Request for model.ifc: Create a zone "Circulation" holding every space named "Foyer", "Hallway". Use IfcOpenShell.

First a look at what the model holds.

```python
import ifcopenshell

model = ifcopenshell.open("model.ifc")
print(model.schema)
seen = {}
for space in model.by_type("IfcSpace"):
    seen[space.LongName] = seen.get(space.LongName, 0) + 1
for name, count in sorted(seen.items(), key=str):
    print(count, "x", name)
print("zones:", [z.Name for z in model.by_type("IfcZone")][:20])
```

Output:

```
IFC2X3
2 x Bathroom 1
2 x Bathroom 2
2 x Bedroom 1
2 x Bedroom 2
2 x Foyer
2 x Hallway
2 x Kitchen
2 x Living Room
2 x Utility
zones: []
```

```python
import ifcopenshell
import ifcopenshell.api.group
import ifcopenshell.api.root

model = ifcopenshell.open("model.ifc")

names = {"Foyer", "Hallway"}
spaces = [s for s in model.by_type("IfcSpace") if s.LongName in names]

zone = ifcopenshell.api.root.create_entity(model, ifc_class="IfcZone", name="Circulation")
ifcopenshell.api.group.assign_group(model, products=spaces, group=zone)
print(len(spaces), "spaces in", zone.Name)

model.write("model_v2.ifc")
```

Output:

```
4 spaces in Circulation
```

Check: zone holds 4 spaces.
